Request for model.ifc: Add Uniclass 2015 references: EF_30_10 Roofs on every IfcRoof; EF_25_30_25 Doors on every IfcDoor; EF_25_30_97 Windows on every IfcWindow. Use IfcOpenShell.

First a look at what the model holds.

```python
import ifcopenshell

model = ifcopenshell.open("model.ifc")
print(model.schema)
print("classifications:", [c.Name for c in model.by_type("IfcClassification")])
for ifc_class in ("IfcDoor", "IfcRoof", "IfcStair", "IfcWall", "IfcWindow"):
    print(ifc_class, len(model.by_type(ifc_class)))
```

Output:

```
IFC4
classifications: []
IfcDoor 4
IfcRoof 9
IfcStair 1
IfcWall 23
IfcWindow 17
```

```python
import ifcopenshell
import ifcopenshell.api.classification

model = ifcopenshell.open("model.ifc")

system = ifcopenshell.api.classification.add_classification(model, classification="Uniclass 2015")

codes = {
    "IfcRoof": ("EF_30_10", "Roofs"),
    "IfcDoor": ("EF_25_30_25", "Doors"),
    "IfcWindow": ("EF_25_30_97", "Windows"),
}
for ifc_class, (code, name) in codes.items():
    products = model.by_type(ifc_class)
    ifcopenshell.api.classification.add_reference(
        model, products=products, classification=system, identification=code, name=name
    )
    print(code, len(products))

model.write("model_edited.ifc")
```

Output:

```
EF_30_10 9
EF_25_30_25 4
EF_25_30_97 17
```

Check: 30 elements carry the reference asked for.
